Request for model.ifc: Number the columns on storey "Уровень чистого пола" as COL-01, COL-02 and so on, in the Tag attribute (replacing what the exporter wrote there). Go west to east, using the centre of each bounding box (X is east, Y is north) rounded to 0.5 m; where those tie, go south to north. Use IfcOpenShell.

First a look at what the model holds.

```python
import ifcopenshell
import ifcopenshell.util.element
import ifcopenshell.util.placement

model = ifcopenshell.open("model.ifc")
print(model.schema)
storey = next(s for s in model.by_type("IfcBuildingStorey") if s.Name == "Уровень чистого пола")
columns = [e for e in ifcopenshell.util.element.get_decomposition(storey) if e.is_a("IfcColumn")]
for e in sorted(columns, key=lambda e: e.id()):
    origin = ifcopenshell.util.placement.get_local_placement(e.ObjectPlacement)[:3, 3]
    print(e.id(), e.Tag, e.Name, origin.round(2) + 0.0, sep=" | ")
```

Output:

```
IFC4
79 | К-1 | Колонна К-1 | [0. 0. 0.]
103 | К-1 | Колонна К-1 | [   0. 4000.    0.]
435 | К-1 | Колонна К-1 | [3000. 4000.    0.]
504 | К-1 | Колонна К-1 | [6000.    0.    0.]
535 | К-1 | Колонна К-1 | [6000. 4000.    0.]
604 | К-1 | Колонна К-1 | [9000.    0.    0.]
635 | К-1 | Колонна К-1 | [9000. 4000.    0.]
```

```python
import ifcopenshell
import ifcopenshell.geom
import ifcopenshell.util.element
import ifcopenshell.util.shape

model = ifcopenshell.open("model.ifc")
settings = ifcopenshell.geom.settings()
settings.set("use-world-coords", True)


def centre(element):
    shape = ifcopenshell.geom.create_shape(settings, element)
    return ifcopenshell.util.shape.get_bbox_centroid(shape.geometry)


storey = next(s for s in model.by_type("IfcBuildingStorey") if s.Name == "Уровень чистого пола")
columns = [e for e in ifcopenshell.util.element.get_decomposition(storey) if e.is_a("IfcColumn")]

# Insertion points can sit at a corner or the storey origin, so sort by the geometry (in metres).
centres = {e: centre(e) for e in columns}
columns.sort(key=lambda e: (round(centres[e][0] / 0.5), centres[e][1]))

for i, e in enumerate(columns, start=1):
    number = f"COL-{i:02d}"
    e.Tag = number
    print(e.id(), number)

model.write("model_rev.ifc")
```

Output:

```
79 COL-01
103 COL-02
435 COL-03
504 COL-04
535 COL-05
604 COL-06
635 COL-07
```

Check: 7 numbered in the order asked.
